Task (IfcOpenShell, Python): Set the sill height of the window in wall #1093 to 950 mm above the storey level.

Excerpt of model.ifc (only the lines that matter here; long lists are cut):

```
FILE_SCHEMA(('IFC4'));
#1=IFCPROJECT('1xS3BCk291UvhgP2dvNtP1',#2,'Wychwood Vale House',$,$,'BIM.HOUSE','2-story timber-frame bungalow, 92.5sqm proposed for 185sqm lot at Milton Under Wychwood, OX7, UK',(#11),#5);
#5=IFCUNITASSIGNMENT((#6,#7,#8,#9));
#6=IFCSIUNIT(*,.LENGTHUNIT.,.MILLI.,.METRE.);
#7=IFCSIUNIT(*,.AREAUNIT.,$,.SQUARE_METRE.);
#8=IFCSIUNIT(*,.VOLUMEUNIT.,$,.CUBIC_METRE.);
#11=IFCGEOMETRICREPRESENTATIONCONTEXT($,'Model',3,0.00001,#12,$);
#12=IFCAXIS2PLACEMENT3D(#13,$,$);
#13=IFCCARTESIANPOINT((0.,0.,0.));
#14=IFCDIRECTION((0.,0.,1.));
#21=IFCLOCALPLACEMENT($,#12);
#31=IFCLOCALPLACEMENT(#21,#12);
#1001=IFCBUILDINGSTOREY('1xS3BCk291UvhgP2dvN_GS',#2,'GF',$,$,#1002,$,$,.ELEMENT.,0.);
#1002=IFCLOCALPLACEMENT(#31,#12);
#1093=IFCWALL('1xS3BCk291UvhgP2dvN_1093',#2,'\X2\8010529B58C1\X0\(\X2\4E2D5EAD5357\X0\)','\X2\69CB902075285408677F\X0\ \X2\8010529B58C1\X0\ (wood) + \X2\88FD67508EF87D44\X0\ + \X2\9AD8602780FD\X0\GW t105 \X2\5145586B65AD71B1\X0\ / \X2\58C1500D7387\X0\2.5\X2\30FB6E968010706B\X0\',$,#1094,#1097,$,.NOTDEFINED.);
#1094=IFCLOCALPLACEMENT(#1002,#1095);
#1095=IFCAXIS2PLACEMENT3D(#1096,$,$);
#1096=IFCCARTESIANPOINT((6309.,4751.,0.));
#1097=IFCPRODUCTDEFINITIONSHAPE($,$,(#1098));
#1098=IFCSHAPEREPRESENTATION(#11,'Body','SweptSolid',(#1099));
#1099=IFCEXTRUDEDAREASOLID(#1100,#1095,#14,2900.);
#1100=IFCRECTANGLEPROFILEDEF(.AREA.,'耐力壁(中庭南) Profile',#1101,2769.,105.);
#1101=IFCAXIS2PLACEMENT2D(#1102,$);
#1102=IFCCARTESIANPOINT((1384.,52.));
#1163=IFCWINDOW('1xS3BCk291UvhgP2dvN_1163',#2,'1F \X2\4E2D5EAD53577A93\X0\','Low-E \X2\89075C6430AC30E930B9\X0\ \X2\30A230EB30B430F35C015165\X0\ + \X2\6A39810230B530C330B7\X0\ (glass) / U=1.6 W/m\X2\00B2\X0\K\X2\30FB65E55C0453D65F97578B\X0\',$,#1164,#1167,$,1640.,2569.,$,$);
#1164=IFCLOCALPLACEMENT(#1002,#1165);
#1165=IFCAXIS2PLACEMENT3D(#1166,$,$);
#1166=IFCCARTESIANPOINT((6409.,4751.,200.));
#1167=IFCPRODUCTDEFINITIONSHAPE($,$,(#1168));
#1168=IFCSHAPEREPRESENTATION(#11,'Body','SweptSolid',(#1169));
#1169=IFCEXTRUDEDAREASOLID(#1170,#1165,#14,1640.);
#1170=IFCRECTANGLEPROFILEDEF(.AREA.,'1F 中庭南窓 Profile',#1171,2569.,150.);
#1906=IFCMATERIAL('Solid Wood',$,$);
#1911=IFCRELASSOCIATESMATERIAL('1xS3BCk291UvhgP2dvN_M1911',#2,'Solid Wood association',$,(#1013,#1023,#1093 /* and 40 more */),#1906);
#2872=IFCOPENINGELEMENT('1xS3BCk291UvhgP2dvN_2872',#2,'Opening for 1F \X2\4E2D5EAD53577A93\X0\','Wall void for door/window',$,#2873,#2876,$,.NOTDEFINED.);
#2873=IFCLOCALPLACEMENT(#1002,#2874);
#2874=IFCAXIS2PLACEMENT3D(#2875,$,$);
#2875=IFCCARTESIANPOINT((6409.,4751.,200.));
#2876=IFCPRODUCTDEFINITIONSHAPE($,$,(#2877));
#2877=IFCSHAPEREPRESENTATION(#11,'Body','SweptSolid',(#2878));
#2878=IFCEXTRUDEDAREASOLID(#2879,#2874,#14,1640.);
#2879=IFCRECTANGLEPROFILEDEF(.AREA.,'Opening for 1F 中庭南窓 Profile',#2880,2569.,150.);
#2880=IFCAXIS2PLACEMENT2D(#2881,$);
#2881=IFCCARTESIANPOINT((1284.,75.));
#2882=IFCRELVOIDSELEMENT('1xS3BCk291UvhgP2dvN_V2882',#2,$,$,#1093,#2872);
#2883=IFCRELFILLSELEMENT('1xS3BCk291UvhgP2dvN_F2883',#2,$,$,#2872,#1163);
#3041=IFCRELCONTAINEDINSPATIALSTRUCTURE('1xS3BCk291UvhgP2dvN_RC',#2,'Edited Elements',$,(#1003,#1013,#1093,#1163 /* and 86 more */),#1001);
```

```python
import numpy as np
import ifcopenshell
import ifcopenshell.api.geometry
import ifcopenshell.geom
import ifcopenshell.util.element
import ifcopenshell.util.placement
import ifcopenshell.util.shape
import ifcopenshell.util.unit

model = ifcopenshell.open("model.ifc")
unit_scale = ifcopenshell.util.unit.calculate_unit_scale(model)

window = model.by_guid("1xS3BCk291UvhgP2dvN_1163")
opening = window.FillsVoids[0].RelatingOpeningElement
storey = ifcopenshell.util.element.get_container(window, ifc_class="IfcBuildingStorey")
level = ifcopenshell.util.placement.get_local_placement(storey.ObjectPlacement)[2, 3]

# The opening's origin need not be at the sill, so measure its lowest point.
shape = ifcopenshell.geom.create_shape(ifcopenshell.geom.settings(), opening)
bottom = ifcopenshell.util.shape.get_shape_bottom_elevation(shape, shape.geometry) / unit_scale
dz = level + 950.0 - bottom

shift = np.array([0.0, 0.0, dz])
# The window is not placed relative to its opening, so move both.
for product in (opening, window):
    matrix = ifcopenshell.util.placement.get_local_placement(product.ObjectPlacement)
    matrix[:3, 3] += shift
    ifcopenshell.api.geometry.edit_object_placement(model, product=product, matrix=matrix, is_si=False)

print(f"moved by {dz * unit_scale:+.3f} m")

model.write("model-out.ifc")
```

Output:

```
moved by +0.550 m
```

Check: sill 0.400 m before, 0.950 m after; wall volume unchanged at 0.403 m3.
